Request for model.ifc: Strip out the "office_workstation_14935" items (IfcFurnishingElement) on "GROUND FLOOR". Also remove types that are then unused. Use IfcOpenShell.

First a look at what the model holds.

```python
import ifcopenshell
import ifcopenshell.util.element

model = ifcopenshell.open("model.ifc")
print(model.schema)
storey = next(s for s in model.by_type("IfcBuildingStorey") if s.Name == "GROUND FLOOR")
furniture = [e for e in ifcopenshell.util.element.get_decomposition(storey) if e.is_a("IfcFurnishingElement")]
seen = {}
for e in furniture:
    element_type = ifcopenshell.util.element.get_type(e)
    name = element_type.Name if element_type not in (None, e) else None
    seen[name] = seen.get(name, 0) + 1
for name, count in sorted(seen.items(), key=str):
    print(count, "x", name)
```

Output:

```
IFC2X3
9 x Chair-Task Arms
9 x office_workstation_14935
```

```python
import ifcopenshell
import ifcopenshell.api.root
import ifcopenshell.util.element

model = ifcopenshell.open("model.ifc")

storey = next(s for s in model.by_type("IfcBuildingStorey") if s.Name == "GROUND FLOOR")
furniture = [e for e in ifcopenshell.util.element.get_decomposition(storey) if e.is_a("IfcFurnishingElement")]
targets = [e for e in furniture if (t := ifcopenshell.util.element.get_type(e)) not in (None, e) and t.Name == "office_workstation_14935"]
types = {ifcopenshell.util.element.get_type(e) for e in targets} - {None, *targets}

for e in targets:
    ifcopenshell.api.root.remove_product(model, product=e)
print(len(targets), "removed")

unused = [t for t in types if not ifcopenshell.util.element.get_types(t)]
for t in unused:
    ifcopenshell.api.root.remove_product(model, product=t)
print(len(unused), "unused types removed")

model.write("model-out.ifc")
```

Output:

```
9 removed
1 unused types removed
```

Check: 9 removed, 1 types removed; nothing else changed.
